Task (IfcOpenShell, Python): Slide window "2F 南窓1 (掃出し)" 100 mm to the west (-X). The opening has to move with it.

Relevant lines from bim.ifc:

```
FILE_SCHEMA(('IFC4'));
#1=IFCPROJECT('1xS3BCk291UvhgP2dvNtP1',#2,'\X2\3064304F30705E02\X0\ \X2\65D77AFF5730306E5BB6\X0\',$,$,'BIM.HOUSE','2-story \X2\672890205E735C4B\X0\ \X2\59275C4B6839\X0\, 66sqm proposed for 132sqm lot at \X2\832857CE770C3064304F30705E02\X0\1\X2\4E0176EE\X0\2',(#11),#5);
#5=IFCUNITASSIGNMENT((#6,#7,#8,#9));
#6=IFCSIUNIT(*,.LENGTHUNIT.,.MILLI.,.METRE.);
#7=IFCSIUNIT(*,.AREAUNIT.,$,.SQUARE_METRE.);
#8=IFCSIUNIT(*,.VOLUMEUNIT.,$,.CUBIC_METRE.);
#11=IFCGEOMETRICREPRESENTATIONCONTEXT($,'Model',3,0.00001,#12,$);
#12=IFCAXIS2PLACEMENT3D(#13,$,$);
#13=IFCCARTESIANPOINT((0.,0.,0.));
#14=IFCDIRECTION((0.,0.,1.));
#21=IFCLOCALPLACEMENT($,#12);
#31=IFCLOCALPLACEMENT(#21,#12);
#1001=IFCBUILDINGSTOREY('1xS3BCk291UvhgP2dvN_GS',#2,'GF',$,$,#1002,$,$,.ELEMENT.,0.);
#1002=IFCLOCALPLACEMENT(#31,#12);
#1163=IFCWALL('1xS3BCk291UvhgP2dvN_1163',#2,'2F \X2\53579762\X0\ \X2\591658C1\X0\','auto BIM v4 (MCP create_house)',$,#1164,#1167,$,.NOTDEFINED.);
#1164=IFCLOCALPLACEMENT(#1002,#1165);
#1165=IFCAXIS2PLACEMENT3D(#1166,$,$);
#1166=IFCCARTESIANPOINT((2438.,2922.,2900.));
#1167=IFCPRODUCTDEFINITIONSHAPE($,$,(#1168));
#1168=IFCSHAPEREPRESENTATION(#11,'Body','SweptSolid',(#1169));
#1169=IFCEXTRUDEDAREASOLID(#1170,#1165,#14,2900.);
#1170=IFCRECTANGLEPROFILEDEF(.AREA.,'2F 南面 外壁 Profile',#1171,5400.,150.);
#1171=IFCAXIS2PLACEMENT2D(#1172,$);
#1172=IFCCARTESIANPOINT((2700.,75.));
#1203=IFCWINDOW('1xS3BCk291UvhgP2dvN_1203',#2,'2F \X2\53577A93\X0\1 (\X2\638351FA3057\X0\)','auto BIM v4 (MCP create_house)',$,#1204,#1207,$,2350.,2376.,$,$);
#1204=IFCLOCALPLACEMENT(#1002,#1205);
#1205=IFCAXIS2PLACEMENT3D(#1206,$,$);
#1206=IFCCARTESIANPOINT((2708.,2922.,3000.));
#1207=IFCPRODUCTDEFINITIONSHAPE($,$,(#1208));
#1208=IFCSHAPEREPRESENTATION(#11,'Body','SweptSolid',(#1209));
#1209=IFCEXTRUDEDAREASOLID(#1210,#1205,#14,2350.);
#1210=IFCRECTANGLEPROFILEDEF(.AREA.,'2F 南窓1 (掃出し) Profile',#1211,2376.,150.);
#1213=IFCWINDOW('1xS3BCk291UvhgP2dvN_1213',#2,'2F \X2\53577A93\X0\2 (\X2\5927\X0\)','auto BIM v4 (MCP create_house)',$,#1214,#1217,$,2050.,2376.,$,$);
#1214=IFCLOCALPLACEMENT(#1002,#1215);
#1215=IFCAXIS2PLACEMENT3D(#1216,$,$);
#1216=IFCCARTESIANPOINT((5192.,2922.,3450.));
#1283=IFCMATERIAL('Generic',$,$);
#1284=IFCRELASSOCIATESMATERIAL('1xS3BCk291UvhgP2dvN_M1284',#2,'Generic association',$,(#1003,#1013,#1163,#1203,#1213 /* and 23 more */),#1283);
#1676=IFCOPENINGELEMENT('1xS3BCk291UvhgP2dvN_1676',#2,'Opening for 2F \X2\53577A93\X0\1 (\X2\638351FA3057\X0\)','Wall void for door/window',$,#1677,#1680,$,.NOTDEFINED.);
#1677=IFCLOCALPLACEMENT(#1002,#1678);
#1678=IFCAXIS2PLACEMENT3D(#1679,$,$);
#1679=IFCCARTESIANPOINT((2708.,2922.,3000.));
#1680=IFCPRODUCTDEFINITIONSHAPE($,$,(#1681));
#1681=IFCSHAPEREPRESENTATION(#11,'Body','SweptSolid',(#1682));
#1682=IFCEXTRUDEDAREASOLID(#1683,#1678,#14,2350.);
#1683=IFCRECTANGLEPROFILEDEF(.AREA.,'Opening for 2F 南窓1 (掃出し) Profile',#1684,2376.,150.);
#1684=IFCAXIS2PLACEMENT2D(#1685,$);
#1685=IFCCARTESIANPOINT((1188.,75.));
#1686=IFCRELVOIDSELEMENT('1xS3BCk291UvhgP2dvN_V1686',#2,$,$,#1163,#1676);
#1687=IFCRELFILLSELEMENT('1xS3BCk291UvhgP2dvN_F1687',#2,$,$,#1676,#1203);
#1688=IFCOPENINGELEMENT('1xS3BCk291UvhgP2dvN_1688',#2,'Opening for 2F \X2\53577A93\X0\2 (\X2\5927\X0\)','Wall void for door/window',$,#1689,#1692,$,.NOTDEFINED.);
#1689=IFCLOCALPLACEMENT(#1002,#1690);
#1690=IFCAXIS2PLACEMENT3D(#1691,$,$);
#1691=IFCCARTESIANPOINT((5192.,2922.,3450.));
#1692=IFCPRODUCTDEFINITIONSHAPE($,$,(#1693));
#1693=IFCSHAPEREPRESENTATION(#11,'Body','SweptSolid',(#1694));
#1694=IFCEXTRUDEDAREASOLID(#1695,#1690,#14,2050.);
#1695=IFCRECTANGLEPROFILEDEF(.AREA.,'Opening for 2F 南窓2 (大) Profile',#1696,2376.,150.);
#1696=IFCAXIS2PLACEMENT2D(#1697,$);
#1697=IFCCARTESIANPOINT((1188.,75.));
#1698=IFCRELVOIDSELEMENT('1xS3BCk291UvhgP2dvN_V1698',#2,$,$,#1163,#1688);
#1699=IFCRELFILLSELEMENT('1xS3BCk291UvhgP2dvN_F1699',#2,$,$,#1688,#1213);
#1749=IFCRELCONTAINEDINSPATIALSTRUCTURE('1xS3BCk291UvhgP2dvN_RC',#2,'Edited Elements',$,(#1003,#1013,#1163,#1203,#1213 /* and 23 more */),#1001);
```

```python
import ifcopenshell
import ifcopenshell.api.geometry
import ifcopenshell.util.placement
import ifcopenshell.util.unit

model = ifcopenshell.open("bim.ifc")
unit_scale = ifcopenshell.util.unit.calculate_unit_scale(model)

window = model.by_guid("1xS3BCk291UvhgP2dvN_1203")
opening = window.FillsVoids[0].RelatingOpeningElement
wall = opening.VoidsElements[0].RelatingBuildingElement

wall_matrix = ifcopenshell.util.placement.get_local_placement(wall.ObjectPlacement)
shift = wall_matrix[:3, 0] * -0.1 / unit_scale
before = ifcopenshell.util.placement.get_local_placement(window.ObjectPlacement)[:3, 3].copy()

# The window is not placed relative to its opening, so move both.
for product in (opening, window):
    matrix = ifcopenshell.util.placement.get_local_placement(product.ObjectPlacement)
    matrix[:3, 3] += shift
    ifcopenshell.api.geometry.edit_object_placement(model, product=product, matrix=matrix, is_si=False)

after = ifcopenshell.util.placement.get_local_placement(window.ObjectPlacement)[:3, 3]
print("window moved by", (after - before).round(3) + 0.0)

model.write("bim_edited.ifc")
```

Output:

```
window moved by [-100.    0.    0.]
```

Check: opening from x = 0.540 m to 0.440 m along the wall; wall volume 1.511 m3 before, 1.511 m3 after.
